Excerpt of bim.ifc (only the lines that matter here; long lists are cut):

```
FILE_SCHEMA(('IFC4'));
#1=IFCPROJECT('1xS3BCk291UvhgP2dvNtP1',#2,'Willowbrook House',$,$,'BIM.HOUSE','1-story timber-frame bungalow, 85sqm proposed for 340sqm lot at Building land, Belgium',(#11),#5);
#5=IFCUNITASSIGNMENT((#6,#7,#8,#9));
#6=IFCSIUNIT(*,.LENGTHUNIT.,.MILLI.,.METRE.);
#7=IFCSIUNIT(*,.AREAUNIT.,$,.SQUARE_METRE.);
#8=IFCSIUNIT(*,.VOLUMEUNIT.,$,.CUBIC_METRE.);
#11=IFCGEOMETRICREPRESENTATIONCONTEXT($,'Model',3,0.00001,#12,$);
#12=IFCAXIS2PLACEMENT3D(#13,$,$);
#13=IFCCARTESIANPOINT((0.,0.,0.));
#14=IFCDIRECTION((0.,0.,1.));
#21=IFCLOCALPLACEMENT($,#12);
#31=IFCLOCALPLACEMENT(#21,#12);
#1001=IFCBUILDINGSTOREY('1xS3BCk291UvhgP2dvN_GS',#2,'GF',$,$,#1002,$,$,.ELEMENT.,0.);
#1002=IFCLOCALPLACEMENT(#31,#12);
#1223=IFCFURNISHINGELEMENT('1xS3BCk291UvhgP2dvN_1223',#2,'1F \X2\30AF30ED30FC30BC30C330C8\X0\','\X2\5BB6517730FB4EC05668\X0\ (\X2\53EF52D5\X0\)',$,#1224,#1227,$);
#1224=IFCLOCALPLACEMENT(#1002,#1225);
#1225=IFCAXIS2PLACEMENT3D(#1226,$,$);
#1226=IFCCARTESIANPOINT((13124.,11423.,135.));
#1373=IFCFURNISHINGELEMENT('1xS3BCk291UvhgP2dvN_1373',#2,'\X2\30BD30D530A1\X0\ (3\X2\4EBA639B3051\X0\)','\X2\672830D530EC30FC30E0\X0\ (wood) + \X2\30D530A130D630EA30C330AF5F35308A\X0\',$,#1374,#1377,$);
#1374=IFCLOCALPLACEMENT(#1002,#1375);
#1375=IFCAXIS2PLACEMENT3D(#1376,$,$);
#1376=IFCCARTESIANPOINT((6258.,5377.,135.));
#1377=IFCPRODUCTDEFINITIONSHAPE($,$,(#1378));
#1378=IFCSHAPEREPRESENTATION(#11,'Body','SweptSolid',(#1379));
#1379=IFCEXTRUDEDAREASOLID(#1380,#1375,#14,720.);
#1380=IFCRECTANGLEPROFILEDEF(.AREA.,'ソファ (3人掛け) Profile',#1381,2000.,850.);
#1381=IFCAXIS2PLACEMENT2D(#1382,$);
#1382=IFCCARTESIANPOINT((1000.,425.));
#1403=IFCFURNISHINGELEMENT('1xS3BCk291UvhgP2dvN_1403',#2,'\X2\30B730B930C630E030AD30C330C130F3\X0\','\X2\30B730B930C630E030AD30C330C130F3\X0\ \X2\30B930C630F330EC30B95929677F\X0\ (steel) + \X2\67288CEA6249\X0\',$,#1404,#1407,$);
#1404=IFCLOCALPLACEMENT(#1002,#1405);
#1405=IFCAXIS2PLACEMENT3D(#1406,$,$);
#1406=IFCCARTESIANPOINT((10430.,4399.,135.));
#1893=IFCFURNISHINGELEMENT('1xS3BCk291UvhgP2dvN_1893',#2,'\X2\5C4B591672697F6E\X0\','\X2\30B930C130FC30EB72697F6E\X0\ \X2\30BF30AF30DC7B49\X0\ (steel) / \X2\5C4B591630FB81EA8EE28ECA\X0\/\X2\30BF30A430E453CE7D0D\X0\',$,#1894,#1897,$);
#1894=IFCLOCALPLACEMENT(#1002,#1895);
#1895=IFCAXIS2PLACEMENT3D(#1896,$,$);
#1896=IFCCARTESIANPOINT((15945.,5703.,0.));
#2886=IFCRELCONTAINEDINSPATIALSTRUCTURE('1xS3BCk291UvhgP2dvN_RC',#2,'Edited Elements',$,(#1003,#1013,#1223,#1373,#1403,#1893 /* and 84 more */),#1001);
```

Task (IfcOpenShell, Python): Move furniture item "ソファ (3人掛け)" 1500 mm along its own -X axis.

```python
import ifcopenshell
import ifcopenshell.api.geometry
import ifcopenshell.util.placement
import ifcopenshell.util.unit

model = ifcopenshell.open("bim.ifc")
unit_scale = ifcopenshell.util.unit.calculate_unit_scale(model)

item = model.by_id(1373)
matrix = ifcopenshell.util.placement.get_local_placement(item.ObjectPlacement)
matrix[:3, 3] -= matrix[:3, 0] * 1.5 / unit_scale
ifcopenshell.api.geometry.edit_object_placement(model, product=item, matrix=matrix, is_si=False)

print(ifcopenshell.util.placement.get_local_placement(item.ObjectPlacement).round(3) + 0.0)

model.write("bim_edited.ifc")
```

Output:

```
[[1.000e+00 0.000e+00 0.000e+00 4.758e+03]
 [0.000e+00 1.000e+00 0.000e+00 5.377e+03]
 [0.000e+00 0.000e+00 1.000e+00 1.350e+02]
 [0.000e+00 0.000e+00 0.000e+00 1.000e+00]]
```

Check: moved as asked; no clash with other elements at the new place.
